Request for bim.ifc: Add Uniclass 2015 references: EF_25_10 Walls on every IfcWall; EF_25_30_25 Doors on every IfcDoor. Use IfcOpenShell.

First a look at what the model holds.

```python
import ifcopenshell

model = ifcopenshell.open("bim.ifc")
print(model.schema)
print("classifications:", [c.Name for c in model.by_type("IfcClassification")])
for ifc_class in ("IfcDoor", "IfcRoof", "IfcStair", "IfcWall", "IfcWindow"):
    print(ifc_class, len(model.by_type(ifc_class)))
```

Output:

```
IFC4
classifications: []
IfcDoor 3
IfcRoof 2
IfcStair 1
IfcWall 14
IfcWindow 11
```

```python
import ifcopenshell
import ifcopenshell.api.classification

model = ifcopenshell.open("bim.ifc")

system = ifcopenshell.api.classification.add_classification(model, classification="Uniclass 2015")

codes = {
    "IfcWall": ("EF_25_10", "Walls"),
    "IfcDoor": ("EF_25_30_25", "Doors"),
}
for ifc_class, (code, name) in codes.items():
    products = model.by_type(ifc_class)
    ifcopenshell.api.classification.add_reference(
        model, products=products, classification=system, identification=code, name=name
    )
    print(code, len(products))

model.write("bim_edited.ifc")
```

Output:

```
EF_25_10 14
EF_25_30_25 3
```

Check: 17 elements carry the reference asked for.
